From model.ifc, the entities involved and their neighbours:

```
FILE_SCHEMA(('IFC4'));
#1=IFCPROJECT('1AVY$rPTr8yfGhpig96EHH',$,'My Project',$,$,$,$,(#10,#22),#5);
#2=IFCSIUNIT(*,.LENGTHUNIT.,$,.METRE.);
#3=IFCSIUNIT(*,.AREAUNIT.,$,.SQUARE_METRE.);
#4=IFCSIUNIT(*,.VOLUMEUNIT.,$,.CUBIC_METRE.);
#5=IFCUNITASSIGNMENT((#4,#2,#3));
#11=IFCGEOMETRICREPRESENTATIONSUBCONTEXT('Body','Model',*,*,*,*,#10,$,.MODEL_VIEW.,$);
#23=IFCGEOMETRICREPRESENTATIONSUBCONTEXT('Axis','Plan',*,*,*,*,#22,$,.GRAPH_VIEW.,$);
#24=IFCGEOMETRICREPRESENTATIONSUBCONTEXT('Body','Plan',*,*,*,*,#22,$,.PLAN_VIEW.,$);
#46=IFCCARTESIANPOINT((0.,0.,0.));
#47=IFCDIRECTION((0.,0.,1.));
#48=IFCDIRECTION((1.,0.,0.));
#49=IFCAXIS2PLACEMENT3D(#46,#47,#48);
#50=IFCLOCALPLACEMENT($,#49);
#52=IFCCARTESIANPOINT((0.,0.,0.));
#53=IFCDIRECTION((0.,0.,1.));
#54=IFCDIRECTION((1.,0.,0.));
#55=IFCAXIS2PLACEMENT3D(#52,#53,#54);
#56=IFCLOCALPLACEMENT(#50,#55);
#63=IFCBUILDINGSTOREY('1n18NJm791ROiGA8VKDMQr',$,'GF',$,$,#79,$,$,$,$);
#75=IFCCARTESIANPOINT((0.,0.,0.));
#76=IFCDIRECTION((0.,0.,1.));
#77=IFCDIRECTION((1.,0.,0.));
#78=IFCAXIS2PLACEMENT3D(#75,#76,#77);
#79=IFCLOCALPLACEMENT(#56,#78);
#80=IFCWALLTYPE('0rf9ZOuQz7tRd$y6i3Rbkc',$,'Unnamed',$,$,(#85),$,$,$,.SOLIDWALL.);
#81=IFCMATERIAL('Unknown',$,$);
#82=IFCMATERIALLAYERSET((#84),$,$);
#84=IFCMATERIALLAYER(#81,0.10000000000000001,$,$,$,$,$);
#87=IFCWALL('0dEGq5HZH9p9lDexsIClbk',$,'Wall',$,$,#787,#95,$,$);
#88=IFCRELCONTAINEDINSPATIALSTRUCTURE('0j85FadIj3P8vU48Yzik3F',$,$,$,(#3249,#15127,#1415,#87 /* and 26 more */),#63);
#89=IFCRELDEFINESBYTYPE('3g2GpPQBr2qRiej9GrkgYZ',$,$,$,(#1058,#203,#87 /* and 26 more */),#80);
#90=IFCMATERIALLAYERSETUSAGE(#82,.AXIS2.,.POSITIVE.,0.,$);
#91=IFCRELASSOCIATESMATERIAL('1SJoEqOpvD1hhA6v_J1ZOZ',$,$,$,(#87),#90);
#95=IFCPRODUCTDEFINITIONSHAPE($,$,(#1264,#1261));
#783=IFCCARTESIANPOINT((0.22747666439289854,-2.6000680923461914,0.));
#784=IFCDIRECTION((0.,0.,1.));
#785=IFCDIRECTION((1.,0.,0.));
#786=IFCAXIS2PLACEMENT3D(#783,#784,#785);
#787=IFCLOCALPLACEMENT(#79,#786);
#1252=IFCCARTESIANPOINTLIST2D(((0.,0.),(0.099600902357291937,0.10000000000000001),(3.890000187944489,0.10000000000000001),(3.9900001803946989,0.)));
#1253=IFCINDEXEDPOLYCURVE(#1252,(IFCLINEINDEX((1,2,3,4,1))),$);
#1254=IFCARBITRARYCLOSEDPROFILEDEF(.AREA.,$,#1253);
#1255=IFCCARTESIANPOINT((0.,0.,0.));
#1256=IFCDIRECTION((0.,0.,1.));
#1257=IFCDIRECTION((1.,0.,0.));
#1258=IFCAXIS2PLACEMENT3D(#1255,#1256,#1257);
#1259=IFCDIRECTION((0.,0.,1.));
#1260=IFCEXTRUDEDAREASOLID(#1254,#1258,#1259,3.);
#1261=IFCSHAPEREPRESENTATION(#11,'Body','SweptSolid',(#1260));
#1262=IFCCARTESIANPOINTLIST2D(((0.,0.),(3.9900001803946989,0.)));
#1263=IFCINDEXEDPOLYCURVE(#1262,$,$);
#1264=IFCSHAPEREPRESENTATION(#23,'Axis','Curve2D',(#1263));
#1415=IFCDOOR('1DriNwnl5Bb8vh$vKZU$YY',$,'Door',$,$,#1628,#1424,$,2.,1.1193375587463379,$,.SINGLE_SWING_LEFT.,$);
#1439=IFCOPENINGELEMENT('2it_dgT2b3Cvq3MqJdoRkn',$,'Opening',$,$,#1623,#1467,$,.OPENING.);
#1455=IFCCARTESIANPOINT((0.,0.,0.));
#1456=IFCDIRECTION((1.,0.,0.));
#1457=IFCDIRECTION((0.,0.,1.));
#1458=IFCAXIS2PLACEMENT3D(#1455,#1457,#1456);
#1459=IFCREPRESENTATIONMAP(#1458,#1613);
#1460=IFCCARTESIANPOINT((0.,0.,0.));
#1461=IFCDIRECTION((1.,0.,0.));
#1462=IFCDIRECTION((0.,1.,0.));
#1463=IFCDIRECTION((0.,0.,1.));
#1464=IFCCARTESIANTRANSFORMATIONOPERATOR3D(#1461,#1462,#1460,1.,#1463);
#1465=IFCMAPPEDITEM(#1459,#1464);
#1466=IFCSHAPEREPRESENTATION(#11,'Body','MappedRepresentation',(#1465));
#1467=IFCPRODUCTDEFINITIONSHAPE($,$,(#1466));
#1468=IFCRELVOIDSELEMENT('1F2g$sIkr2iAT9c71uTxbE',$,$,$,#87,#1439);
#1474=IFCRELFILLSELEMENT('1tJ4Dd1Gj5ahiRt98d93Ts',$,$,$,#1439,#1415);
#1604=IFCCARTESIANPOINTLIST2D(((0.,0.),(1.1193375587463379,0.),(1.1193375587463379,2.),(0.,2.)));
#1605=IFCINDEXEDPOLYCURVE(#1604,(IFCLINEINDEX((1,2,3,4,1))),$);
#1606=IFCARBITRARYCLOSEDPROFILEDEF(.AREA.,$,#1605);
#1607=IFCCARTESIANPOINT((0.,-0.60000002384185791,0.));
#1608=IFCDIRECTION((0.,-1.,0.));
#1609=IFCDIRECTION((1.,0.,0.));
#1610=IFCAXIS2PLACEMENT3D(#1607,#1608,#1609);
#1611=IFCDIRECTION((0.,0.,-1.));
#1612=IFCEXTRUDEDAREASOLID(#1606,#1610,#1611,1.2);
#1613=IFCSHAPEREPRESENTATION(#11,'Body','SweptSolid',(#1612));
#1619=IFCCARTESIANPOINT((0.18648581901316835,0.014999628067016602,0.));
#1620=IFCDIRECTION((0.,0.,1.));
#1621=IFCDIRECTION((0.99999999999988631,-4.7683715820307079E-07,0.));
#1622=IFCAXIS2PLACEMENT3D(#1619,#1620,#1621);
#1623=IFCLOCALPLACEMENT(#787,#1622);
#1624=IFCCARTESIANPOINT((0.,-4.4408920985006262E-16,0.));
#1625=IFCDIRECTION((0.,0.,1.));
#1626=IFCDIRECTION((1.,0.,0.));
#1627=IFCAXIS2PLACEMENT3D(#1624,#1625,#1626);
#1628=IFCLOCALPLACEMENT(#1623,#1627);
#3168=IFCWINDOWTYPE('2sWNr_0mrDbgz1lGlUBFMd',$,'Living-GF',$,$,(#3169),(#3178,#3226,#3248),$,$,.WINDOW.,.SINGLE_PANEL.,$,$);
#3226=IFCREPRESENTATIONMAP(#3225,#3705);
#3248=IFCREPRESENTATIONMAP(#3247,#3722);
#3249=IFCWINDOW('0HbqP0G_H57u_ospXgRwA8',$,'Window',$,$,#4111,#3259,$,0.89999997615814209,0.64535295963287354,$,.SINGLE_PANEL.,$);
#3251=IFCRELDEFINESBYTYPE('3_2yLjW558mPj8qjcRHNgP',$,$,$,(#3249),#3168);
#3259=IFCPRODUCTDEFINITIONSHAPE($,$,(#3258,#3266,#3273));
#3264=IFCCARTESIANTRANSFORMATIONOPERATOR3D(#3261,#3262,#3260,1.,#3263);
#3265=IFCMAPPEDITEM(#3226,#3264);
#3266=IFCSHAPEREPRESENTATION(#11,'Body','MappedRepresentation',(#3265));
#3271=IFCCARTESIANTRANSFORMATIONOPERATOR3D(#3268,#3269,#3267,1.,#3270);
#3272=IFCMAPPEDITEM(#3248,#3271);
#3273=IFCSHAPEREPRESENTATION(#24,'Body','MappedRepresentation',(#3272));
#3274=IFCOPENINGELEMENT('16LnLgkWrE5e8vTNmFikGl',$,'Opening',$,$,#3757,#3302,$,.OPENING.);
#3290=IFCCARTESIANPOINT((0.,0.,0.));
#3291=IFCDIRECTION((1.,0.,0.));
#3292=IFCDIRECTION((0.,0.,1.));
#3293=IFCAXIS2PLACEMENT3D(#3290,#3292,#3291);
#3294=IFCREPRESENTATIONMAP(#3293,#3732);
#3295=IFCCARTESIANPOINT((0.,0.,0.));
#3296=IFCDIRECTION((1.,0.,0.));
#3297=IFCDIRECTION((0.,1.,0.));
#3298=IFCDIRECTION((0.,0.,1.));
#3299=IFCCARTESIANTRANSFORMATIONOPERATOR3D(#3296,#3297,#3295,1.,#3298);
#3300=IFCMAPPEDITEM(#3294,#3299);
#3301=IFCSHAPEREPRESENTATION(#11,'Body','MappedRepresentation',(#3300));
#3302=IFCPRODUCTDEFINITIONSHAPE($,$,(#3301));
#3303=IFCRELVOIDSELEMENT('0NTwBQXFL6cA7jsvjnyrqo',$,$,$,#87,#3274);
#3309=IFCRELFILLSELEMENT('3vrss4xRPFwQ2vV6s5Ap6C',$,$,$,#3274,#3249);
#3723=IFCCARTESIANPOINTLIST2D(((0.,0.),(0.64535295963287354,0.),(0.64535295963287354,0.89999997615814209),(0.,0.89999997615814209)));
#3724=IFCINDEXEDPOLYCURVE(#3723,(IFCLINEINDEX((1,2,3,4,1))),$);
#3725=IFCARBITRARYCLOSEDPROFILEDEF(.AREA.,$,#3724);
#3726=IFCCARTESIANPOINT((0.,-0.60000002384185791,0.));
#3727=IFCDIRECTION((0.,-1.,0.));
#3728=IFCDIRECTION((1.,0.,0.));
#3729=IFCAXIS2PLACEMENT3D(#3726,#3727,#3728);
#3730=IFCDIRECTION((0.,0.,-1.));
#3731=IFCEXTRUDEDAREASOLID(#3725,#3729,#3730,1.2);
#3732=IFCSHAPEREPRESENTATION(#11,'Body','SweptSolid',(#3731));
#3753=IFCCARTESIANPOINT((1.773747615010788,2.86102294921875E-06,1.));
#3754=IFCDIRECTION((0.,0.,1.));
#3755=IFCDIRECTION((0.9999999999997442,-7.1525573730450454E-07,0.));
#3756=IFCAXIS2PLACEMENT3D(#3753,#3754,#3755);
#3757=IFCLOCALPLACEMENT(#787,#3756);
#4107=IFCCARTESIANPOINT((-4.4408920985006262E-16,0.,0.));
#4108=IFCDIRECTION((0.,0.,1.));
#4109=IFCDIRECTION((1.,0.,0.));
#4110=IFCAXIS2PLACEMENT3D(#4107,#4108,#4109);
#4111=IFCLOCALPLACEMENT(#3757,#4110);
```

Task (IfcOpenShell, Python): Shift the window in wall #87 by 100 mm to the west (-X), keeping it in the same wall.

```python
import ifcopenshell
import ifcopenshell.api.geometry
import ifcopenshell.util.placement

model = ifcopenshell.open("model.ifc")

window = model.by_id(3249)
opening = window.FillsVoids[0].RelatingOpeningElement
wall = opening.VoidsElements[0].RelatingBuildingElement

wall_matrix = ifcopenshell.util.placement.get_local_placement(wall.ObjectPlacement)
shift = wall_matrix[:3, 0] * -0.1
before = ifcopenshell.util.placement.get_local_placement(window.ObjectPlacement)[:3, 3].copy()

# The window is placed relative to its opening, so it follows when the opening moves.
matrix = ifcopenshell.util.placement.get_local_placement(opening.ObjectPlacement)
matrix[:3, 3] += shift
ifcopenshell.api.geometry.edit_object_placement(
    model, product=opening, matrix=matrix, is_si=False, should_transform_children=True
)

after = ifcopenshell.util.placement.get_local_placement(window.ObjectPlacement)[:3, 3]
print("window moved by", (after - before).round(3) + 0.0)

model.write("model-out.ifc")
```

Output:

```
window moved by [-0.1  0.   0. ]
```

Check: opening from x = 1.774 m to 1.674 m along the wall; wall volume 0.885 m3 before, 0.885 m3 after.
